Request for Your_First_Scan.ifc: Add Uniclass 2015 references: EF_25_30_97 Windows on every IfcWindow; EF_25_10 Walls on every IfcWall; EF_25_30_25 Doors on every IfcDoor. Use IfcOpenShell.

First a look at what the model holds.

```python
import ifcopenshell

model = ifcopenshell.open("Your_First_Scan.ifc")
print(model.schema)
print("classifications:", [c.Name for c in model.by_type("IfcClassification")])
for ifc_class in ("IfcDoor", "IfcRoof", "IfcStair", "IfcWall", "IfcWindow"):
    print(ifc_class, len(model.by_type(ifc_class)))
```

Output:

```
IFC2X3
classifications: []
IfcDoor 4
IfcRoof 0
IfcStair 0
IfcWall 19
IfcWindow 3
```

```python
import ifcopenshell
import ifcopenshell.api.classification

model = ifcopenshell.open("Your_First_Scan.ifc")

# IFC2X3 requires Source and Edition and has no link from the project to the system.
system = model.create_entity("IfcClassification", Source="NBS", Edition="2015", Name="Uniclass 2015")

codes = {
    "IfcWindow": ("EF_25_30_97", "Windows"),
    "IfcWall": ("EF_25_10", "Walls"),
    "IfcDoor": ("EF_25_30_25", "Doors"),
}
for ifc_class, (code, name) in codes.items():
    products = model.by_type(ifc_class)
    ifcopenshell.api.classification.add_reference(
        model, products=products, classification=system, identification=code, name=name
    )
    print(code, len(products))

model.write("Your_First_Scan_v2.ifc")
```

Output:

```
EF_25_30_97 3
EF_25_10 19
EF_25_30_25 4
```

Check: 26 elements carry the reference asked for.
